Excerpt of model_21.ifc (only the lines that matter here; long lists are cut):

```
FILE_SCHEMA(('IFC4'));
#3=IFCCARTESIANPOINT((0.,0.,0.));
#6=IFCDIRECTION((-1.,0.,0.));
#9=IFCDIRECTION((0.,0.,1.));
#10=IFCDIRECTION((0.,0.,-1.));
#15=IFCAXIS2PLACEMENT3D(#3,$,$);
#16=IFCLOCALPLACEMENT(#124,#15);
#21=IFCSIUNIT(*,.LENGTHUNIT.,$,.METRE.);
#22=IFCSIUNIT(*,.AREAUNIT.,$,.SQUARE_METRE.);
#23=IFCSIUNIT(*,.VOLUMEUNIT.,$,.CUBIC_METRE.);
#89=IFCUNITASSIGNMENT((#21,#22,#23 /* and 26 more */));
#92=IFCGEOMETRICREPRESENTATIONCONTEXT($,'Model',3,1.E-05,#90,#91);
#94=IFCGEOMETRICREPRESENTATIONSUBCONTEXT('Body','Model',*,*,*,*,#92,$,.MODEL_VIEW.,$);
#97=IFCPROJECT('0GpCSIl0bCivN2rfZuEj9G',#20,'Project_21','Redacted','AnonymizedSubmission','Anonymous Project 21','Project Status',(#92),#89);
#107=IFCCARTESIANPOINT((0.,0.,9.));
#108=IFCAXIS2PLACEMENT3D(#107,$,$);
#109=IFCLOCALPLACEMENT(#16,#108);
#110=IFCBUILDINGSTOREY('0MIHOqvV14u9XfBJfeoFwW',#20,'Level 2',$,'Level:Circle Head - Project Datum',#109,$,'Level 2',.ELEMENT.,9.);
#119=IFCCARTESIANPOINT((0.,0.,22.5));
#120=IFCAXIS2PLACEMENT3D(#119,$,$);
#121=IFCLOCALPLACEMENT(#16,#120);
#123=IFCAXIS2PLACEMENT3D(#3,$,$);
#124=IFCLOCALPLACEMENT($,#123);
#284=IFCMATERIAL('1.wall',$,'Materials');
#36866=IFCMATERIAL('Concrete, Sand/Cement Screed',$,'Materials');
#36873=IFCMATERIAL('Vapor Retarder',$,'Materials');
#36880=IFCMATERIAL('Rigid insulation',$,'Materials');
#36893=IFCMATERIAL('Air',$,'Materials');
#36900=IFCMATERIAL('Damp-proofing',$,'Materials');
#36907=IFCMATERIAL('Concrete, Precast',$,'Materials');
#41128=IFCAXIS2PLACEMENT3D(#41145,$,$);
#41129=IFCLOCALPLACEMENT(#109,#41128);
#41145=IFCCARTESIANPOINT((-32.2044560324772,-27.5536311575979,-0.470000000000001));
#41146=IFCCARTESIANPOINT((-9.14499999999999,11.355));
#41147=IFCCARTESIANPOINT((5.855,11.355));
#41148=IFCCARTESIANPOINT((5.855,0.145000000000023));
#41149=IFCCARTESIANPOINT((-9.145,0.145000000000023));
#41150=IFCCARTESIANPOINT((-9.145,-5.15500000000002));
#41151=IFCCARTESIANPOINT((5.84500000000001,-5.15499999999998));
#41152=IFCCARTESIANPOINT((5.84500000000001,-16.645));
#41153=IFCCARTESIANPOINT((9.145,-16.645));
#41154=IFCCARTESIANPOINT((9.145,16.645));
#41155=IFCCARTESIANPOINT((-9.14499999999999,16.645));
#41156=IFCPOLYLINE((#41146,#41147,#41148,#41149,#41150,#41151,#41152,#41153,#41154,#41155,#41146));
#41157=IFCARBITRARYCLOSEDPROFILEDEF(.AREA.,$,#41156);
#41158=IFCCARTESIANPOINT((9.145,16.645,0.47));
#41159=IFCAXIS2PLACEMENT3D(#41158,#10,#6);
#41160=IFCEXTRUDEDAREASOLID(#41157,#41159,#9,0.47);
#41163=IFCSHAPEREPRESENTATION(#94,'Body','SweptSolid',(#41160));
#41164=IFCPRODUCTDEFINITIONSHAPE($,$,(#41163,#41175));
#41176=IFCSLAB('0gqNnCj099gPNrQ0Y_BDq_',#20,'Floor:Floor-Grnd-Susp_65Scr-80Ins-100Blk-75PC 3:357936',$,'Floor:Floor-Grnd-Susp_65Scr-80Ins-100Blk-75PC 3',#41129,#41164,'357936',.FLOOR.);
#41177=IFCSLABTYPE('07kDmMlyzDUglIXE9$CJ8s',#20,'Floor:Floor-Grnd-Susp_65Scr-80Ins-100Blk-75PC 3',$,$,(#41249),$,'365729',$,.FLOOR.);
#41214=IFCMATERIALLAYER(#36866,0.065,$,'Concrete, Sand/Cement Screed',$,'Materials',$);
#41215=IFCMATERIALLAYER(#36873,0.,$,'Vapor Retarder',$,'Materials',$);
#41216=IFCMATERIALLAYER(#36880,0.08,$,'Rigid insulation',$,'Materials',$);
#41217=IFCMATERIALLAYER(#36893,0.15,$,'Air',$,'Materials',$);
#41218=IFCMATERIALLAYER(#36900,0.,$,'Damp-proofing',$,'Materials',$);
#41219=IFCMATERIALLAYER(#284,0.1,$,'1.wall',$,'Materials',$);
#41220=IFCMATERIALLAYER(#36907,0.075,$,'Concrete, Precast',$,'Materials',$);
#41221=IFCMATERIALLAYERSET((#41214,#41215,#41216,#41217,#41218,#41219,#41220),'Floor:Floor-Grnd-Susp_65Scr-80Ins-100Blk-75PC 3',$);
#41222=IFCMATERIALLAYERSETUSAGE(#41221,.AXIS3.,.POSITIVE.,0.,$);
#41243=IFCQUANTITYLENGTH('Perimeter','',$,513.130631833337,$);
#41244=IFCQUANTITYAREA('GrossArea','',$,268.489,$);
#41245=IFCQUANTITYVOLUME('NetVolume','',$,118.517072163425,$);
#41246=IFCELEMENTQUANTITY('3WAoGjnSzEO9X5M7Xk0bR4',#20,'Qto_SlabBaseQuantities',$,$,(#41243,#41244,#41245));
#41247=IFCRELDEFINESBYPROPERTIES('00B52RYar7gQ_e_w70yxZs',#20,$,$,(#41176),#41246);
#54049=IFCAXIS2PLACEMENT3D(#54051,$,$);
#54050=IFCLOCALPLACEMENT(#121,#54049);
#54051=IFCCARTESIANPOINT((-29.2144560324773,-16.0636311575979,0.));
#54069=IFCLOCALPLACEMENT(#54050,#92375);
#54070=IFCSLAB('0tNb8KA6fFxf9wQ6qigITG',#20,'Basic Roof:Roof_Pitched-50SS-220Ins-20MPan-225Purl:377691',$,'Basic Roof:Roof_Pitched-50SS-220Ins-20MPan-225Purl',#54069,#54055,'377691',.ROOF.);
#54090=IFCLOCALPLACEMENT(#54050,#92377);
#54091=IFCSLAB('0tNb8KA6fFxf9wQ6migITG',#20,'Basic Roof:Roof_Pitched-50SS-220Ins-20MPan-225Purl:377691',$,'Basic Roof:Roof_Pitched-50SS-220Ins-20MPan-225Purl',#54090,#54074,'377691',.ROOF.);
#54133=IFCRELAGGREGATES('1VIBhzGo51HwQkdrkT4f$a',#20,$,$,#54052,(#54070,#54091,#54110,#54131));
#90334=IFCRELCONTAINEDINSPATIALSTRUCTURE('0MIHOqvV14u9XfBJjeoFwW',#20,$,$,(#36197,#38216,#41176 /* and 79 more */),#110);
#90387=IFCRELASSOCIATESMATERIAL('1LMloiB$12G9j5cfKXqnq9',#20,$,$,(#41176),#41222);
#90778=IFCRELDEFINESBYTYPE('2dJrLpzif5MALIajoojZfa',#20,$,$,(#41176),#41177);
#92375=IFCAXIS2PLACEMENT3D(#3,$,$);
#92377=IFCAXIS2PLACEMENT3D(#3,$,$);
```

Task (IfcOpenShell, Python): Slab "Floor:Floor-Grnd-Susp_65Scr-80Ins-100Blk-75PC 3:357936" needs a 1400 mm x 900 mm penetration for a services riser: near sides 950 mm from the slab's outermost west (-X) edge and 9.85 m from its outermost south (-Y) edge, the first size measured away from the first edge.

```python
import numpy as np
import ifcopenshell
import ifcopenshell.api.feature
import ifcopenshell.api.geometry
import ifcopenshell.api.pset
import ifcopenshell.api.root
import ifcopenshell.geom
import ifcopenshell.util.element
import ifcopenshell.util.placement
import ifcopenshell.util.representation
import ifcopenshell.util.shape
import ifcopenshell.util.unit

model = ifcopenshell.open("model_21.ifc")
unit_scale = ifcopenshell.util.unit.calculate_unit_scale(model)
volume_scale = ifcopenshell.util.unit.calculate_unit_scale(model, "VOLUMEUNIT")
settings = ifcopenshell.geom.settings()


def volume(element):
    """Net volume in cubic metres, openings subtracted."""
    shape = ifcopenshell.geom.create_shape(settings, element)
    return ifcopenshell.util.shape.get_volume(shape.geometry)


slab = model.by_id(41176)
before = volume(slab)

# Extent in the slab's own axes, in metres. The edges named are its -X and -Y sides.
slab_shape = ifcopenshell.geom.create_shape(settings, slab)
vertices = ifcopenshell.util.shape.get_vertices(slab_shape.geometry)
x_min, y_min, bottom = vertices.min(axis=0)
top = vertices[:, 2].max()

opening = ifcopenshell.api.root.create_entity(model, ifc_class="IfcOpeningElement", name="Services riser opening", predefined_type="OPENING")
context = ifcopenshell.util.representation.get_context(model, "Model", "Body", "MODEL_VIEW")
width, depth = 1.4, 0.9
outline = [(0.0, 0.0), (width, 0.0), (width, depth), (0.0, depth), (0.0, 0.0)]
# Overshoot both faces by 50 mm so the cut is clean.
shape = ifcopenshell.api.geometry.add_slab_representation(
    model, context=context, depth=top - bottom + 0.1, polyline=outline
)
ifcopenshell.api.geometry.assign_representation(model, product=opening, representation=shape)

matrix = ifcopenshell.util.placement.get_local_placement(slab.ObjectPlacement)
matrix[:, 3] = matrix @ np.append(np.array([x_min + 0.95, y_min + 9.85, bottom - 0.05]) / unit_scale, 1.0)
ifcopenshell.api.geometry.edit_object_placement(model, product=opening, matrix=matrix, is_si=False)
ifcopenshell.api.feature.add_feature(model, feature=opening, element=slab)

after = volume(slab)

# Update the slab's stored quantities.
qto = model.by_id(ifcopenshell.util.element.get_pset(slab, "Qto_SlabBaseQuantities", should_inherit=False)["id"])
ifcopenshell.api.pset.edit_qto(model, qto=qto, properties={"NetVolume": after / volume_scale})

print(f"slab volume {before:.3f} -> {after:.3f} m3")

model.write("model_21_v2.ifc")
```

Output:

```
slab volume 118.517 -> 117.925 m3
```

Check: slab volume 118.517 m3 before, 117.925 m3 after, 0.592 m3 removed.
